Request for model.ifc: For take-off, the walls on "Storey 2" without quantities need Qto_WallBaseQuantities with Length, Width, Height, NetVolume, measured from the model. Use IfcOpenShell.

First a look at what the model holds.

```python
import ifcopenshell
import ifcopenshell.util.element
import ifcopenshell.util.unit

model = ifcopenshell.open("model.ifc")
print(model.schema)
for unit_type in ("LENGTHUNIT", "AREAUNIT", "VOLUMEUNIT"):
    print(unit_type, ifcopenshell.util.unit.calculate_unit_scale(model, unit_type))
storey = next(s for s in model.by_type("IfcBuildingStorey") if s.Name == "Storey 2")
walls = [e for e in ifcopenshell.util.element.get_decomposition(storey) if e.is_a("IfcWall")]
for e in sorted(walls, key=lambda e: e.id()):
    print(e.id(), e.is_a(), e.Name, list(ifcopenshell.util.element.get_psets(e, qtos_only=True)), sep=" | ")
```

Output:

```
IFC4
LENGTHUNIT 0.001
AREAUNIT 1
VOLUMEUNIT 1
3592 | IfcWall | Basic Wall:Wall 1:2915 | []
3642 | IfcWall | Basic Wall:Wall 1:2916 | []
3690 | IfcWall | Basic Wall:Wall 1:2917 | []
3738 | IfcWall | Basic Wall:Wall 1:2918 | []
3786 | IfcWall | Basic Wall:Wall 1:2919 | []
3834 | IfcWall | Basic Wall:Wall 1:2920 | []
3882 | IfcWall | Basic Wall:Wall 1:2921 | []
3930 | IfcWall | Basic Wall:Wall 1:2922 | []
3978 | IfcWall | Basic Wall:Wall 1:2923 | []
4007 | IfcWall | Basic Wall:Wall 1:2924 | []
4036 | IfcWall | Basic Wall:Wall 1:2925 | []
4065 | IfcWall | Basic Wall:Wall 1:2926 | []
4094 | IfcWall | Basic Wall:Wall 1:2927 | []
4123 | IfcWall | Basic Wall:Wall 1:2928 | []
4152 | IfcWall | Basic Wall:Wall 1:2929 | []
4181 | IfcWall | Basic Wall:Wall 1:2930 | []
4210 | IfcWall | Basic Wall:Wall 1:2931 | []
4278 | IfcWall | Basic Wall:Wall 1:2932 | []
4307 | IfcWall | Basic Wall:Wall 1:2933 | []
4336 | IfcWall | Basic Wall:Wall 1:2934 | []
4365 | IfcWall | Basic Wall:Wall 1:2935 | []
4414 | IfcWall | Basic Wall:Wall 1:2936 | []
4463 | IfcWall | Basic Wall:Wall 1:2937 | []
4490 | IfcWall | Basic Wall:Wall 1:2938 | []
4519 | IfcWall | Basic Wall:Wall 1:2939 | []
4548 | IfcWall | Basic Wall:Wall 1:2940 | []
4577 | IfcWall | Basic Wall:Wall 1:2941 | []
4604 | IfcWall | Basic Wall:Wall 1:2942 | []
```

```python
import ifcopenshell
import ifcopenshell.api.pset
import ifcopenshell.geom
import ifcopenshell.util.element
import ifcopenshell.util.shape
import ifcopenshell.util.unit

model = ifcopenshell.open("model.ifc")
unit_scale = ifcopenshell.util.unit.calculate_unit_scale(model)
volume_scale = ifcopenshell.util.unit.calculate_unit_scale(model, "VOLUMEUNIT")
settings = ifcopenshell.geom.settings()

storey = next(s for s in model.by_type("IfcBuildingStorey") if s.Name == "Storey 2")
walls = [e for e in ifcopenshell.util.element.get_decomposition(storey) if e.is_a("IfcWall")]

for e in sorted(walls, key=lambda e: e.id()):
    if ifcopenshell.util.element.get_psets(e, qtos_only=True, should_inherit=False):
        continue
    # Geometry comes back in metres, in the element's own axes.
    shape = ifcopenshell.geom.create_shape(settings, e)
    values = {
        "Length": ifcopenshell.util.shape.get_x(shape.geometry) / unit_scale,
        "Width": ifcopenshell.util.shape.get_y(shape.geometry) / unit_scale,
        "Height": ifcopenshell.util.shape.get_z(shape.geometry) / unit_scale,
        "NetVolume": ifcopenshell.util.shape.get_volume(shape.geometry) / volume_scale,
    }
    qto = ifcopenshell.api.pset.add_qto(model, product=e, name="Qto_WallBaseQuantities")
    ifcopenshell.api.pset.edit_qto(model, qto=qto, properties=values)
    print(e.id(), {k: round(v, 3) for k, v in values.items()})

model.write("model_v2.ifc")
```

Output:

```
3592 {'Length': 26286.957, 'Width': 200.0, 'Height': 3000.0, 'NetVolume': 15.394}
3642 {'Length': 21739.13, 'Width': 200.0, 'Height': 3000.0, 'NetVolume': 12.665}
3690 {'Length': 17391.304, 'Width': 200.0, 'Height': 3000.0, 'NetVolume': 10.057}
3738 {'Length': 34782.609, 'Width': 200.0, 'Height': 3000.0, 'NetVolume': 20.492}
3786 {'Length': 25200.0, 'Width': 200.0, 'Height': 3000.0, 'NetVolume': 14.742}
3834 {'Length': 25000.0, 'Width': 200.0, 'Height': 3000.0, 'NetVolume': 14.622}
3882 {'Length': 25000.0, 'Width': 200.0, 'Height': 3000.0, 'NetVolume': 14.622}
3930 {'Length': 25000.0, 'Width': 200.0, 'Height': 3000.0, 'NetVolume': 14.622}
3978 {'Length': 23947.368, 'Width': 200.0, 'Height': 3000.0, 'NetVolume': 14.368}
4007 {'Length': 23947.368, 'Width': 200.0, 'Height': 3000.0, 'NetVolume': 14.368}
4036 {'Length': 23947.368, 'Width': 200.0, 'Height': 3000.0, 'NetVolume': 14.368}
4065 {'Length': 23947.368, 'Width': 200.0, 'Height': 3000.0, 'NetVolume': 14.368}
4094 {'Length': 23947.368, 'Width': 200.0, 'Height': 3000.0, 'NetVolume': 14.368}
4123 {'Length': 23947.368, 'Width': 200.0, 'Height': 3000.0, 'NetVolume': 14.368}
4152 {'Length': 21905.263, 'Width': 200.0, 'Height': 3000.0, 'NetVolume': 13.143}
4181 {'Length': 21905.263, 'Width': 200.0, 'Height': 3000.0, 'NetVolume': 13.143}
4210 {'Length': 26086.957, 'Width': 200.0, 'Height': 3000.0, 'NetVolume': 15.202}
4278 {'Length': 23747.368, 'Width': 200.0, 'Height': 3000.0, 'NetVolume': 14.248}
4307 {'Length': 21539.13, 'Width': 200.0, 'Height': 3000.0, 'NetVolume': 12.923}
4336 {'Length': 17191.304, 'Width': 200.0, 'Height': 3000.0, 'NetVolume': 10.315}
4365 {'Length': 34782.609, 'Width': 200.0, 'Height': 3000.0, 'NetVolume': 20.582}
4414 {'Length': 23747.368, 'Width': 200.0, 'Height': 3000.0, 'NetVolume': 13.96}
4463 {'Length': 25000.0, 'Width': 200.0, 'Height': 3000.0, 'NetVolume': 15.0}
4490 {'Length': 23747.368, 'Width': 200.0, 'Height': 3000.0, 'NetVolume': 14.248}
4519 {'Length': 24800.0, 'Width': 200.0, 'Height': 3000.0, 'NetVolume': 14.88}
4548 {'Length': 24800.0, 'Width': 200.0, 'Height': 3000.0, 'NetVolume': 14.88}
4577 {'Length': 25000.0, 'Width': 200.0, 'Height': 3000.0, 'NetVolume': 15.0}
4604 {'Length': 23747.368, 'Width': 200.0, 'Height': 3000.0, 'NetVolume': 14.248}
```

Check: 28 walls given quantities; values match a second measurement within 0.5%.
